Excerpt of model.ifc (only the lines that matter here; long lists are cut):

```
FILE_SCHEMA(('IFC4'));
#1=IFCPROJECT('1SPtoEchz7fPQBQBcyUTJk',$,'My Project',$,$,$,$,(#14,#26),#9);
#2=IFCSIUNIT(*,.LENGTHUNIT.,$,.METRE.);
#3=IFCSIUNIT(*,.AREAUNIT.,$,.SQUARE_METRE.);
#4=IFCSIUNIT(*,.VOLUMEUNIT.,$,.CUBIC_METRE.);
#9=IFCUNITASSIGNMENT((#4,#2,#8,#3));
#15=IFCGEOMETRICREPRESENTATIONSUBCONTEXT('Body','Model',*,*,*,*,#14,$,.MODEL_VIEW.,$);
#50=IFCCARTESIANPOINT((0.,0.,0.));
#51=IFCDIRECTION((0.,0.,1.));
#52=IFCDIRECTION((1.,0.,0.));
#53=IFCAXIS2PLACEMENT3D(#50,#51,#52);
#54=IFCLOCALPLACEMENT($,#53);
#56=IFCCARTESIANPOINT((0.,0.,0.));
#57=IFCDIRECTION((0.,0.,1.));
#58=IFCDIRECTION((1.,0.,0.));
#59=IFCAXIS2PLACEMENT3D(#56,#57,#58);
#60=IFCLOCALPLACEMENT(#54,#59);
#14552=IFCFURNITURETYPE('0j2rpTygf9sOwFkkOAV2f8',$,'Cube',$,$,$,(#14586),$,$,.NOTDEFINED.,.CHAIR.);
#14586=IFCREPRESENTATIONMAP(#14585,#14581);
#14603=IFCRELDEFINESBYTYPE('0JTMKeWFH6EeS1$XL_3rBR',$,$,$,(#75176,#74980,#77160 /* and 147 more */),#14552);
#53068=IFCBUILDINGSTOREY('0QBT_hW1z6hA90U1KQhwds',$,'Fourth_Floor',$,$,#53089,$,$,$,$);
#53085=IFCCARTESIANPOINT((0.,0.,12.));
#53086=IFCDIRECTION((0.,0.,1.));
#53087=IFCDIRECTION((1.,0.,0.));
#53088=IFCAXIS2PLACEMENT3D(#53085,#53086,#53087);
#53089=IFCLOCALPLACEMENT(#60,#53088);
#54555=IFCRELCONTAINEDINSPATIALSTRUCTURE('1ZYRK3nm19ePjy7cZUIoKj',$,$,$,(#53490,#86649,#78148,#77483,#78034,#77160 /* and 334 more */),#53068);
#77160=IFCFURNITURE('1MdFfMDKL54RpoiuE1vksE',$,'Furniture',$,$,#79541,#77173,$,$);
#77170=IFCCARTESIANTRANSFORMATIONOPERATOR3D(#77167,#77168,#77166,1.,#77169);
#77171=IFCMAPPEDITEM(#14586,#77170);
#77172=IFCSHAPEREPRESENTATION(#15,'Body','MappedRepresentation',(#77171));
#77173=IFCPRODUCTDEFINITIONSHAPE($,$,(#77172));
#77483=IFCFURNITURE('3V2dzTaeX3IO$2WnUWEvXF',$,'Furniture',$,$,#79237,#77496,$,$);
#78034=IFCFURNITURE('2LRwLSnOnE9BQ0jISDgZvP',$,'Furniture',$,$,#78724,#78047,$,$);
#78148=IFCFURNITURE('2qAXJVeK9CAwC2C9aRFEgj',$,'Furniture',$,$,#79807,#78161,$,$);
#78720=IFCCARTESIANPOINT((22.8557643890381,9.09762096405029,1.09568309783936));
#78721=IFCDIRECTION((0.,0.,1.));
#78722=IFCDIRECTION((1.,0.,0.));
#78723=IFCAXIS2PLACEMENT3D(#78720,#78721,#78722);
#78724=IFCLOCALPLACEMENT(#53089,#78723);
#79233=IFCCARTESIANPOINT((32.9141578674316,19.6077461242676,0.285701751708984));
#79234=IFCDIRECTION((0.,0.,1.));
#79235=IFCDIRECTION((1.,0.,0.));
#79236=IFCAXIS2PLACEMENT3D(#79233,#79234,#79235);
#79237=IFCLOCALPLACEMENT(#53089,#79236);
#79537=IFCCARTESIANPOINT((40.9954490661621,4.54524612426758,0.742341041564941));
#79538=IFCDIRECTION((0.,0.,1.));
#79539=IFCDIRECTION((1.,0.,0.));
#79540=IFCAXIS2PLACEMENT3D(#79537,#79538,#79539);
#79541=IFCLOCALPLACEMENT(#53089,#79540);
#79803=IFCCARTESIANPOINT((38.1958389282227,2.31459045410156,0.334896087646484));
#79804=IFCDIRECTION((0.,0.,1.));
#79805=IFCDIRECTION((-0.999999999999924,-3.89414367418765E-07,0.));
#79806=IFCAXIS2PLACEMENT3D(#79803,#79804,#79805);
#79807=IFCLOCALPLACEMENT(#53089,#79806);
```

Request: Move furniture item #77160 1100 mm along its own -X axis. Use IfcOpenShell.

```python
import ifcopenshell
import ifcopenshell.api.geometry
import ifcopenshell.util.placement

model = ifcopenshell.open("model.ifc")

item = model.by_id(77160)
matrix = ifcopenshell.util.placement.get_local_placement(item.ObjectPlacement)
matrix[:3, 3] -= matrix[:3, 0] * 1.1
ifcopenshell.api.geometry.edit_object_placement(model, product=item, matrix=matrix, is_si=False)

print(ifcopenshell.util.placement.get_local_placement(item.ObjectPlacement).round(3) + 0.0)

model.write("model_updated.ifc")
```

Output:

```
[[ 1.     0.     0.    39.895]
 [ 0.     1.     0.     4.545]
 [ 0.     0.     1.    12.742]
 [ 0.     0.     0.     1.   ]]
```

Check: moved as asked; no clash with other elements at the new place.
